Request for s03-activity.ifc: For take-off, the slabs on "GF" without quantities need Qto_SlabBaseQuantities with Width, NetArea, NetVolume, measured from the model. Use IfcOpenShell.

First a look at what the model holds.

```python
import ifcopenshell
import ifcopenshell.util.element
import ifcopenshell.util.unit

model = ifcopenshell.open("s03-activity.ifc")
print(model.schema)
for unit_type in ("LENGTHUNIT", "AREAUNIT", "VOLUMEUNIT"):
    print(unit_type, ifcopenshell.util.unit.calculate_unit_scale(model, unit_type))
storey = next(s for s in model.by_type("IfcBuildingStorey") if s.Name == "GF")
slabs = [e for e in ifcopenshell.util.element.get_decomposition(storey) if e.is_a("IfcSlab")]
for e in sorted(slabs, key=lambda e: e.id()):
    print(e.id(), e.is_a(), e.Name, list(ifcopenshell.util.element.get_psets(e, qtos_only=True)), sep=" | ")
```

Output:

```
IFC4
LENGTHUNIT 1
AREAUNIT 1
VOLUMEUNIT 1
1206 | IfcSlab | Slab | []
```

```python
import ifcopenshell
import ifcopenshell.api.pset
import ifcopenshell.geom
import ifcopenshell.util.element
import ifcopenshell.util.shape
import ifcopenshell.util.unit

model = ifcopenshell.open("s03-activity.ifc")
unit_scale = ifcopenshell.util.unit.calculate_unit_scale(model)
area_scale = ifcopenshell.util.unit.calculate_unit_scale(model, "AREAUNIT")
volume_scale = ifcopenshell.util.unit.calculate_unit_scale(model, "VOLUMEUNIT")
settings = ifcopenshell.geom.settings()

storey = next(s for s in model.by_type("IfcBuildingStorey") if s.Name == "GF")
slabs = [e for e in ifcopenshell.util.element.get_decomposition(storey) if e.is_a("IfcSlab")]

for e in sorted(slabs, key=lambda e: e.id()):
    if ifcopenshell.util.element.get_psets(e, qtos_only=True, should_inherit=False):
        continue
    # Geometry comes back in metres, in the element's own axes.
    shape = ifcopenshell.geom.create_shape(settings, e)
    values = {
        "Width": ifcopenshell.util.shape.get_z(shape.geometry) / unit_scale,
        "NetArea": ifcopenshell.util.shape.get_footprint_area(shape.geometry) / area_scale,
        "NetVolume": ifcopenshell.util.shape.get_volume(shape.geometry) / volume_scale,
    }
    qto = ifcopenshell.api.pset.add_qto(model, product=e, name="Qto_SlabBaseQuantities")
    ifcopenshell.api.pset.edit_qto(model, qto=qto, properties=values)
    print(e.id(), {k: round(v, 3) for k, v in values.items()})

model.write("s03-activity_updated.ifc")
```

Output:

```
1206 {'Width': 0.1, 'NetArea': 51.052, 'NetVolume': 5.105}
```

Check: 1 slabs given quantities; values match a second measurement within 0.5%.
